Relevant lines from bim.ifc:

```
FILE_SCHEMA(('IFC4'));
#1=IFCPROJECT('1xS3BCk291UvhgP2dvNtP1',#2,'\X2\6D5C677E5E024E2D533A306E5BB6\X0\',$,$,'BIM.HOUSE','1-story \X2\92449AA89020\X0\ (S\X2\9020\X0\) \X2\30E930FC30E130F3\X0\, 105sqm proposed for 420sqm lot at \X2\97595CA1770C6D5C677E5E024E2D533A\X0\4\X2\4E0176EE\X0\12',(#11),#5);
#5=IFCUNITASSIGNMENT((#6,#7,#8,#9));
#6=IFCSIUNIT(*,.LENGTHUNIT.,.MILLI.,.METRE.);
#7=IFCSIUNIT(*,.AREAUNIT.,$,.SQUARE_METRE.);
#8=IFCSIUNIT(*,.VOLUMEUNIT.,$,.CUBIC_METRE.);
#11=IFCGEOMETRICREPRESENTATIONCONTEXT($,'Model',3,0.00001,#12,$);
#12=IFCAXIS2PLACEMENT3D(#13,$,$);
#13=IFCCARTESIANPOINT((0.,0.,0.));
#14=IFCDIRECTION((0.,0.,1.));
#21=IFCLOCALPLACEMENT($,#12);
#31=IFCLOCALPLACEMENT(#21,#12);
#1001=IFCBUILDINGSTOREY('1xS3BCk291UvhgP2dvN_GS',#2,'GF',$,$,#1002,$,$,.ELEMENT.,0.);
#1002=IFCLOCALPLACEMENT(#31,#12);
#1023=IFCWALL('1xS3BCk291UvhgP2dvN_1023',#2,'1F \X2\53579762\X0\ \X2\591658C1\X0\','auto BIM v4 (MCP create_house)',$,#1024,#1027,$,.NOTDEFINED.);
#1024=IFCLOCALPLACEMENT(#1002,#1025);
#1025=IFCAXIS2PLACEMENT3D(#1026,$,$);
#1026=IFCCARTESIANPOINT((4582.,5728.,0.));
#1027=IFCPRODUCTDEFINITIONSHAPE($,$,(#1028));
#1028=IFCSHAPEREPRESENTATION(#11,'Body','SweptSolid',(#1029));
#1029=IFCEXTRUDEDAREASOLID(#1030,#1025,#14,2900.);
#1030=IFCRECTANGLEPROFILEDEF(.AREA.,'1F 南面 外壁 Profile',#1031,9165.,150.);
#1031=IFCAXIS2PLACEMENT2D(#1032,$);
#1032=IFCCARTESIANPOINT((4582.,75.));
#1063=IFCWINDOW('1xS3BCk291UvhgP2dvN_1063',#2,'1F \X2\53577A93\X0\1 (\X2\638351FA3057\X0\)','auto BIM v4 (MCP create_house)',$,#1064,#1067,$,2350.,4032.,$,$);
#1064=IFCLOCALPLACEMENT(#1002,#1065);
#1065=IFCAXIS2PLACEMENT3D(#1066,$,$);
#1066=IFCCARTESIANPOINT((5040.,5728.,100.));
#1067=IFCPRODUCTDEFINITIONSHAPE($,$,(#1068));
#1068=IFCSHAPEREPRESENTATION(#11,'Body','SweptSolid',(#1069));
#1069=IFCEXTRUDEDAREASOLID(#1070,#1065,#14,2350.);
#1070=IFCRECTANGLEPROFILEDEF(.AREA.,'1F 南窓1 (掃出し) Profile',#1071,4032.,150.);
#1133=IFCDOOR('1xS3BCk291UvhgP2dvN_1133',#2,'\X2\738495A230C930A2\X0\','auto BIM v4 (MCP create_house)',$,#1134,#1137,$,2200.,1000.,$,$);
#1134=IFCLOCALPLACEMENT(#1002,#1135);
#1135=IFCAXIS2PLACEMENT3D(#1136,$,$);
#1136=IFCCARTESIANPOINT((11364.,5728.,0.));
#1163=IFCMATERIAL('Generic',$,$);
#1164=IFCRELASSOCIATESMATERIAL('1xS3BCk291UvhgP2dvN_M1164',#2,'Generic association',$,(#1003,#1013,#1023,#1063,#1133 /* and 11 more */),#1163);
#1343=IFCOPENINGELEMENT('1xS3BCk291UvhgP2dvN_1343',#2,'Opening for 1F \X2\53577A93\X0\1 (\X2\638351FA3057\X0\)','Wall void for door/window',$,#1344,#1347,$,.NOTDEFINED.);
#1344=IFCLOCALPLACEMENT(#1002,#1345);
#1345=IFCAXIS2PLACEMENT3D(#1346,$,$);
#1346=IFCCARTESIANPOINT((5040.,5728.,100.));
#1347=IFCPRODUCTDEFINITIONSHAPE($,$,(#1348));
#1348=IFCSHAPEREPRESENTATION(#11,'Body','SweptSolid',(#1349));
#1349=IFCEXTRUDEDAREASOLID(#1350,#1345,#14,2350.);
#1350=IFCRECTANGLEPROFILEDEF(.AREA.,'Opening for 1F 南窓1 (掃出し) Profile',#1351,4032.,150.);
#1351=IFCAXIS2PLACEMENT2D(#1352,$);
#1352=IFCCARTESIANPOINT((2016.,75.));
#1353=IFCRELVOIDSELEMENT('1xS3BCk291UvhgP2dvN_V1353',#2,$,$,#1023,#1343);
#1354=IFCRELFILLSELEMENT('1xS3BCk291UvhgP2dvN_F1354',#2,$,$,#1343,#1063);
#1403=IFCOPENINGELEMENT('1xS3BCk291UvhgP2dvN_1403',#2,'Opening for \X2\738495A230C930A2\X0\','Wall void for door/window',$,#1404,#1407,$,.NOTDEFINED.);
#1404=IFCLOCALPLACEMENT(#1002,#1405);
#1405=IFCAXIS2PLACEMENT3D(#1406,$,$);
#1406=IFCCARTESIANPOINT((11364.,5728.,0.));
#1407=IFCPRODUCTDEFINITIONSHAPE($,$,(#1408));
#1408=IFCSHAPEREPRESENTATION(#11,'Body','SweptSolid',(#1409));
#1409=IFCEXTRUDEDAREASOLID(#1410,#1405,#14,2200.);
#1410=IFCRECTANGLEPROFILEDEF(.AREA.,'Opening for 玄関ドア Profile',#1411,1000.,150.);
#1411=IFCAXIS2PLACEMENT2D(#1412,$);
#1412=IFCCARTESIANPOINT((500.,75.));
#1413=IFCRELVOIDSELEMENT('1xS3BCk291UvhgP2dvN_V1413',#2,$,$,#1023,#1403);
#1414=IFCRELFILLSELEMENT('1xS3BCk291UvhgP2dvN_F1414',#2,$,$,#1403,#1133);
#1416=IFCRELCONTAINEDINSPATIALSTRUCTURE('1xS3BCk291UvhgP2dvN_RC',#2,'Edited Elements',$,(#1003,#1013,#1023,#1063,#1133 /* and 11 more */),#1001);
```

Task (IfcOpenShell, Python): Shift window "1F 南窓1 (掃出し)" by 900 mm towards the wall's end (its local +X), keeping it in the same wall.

```python
import ifcopenshell
import ifcopenshell.api.geometry
import ifcopenshell.util.placement
import ifcopenshell.util.unit

model = ifcopenshell.open("bim.ifc")
unit_scale = ifcopenshell.util.unit.calculate_unit_scale(model)

window = model.by_id(1063)
opening = window.FillsVoids[0].RelatingOpeningElement
wall = opening.VoidsElements[0].RelatingBuildingElement

wall_matrix = ifcopenshell.util.placement.get_local_placement(wall.ObjectPlacement)
shift = wall_matrix[:3, 0] * 0.9 / unit_scale
before = ifcopenshell.util.placement.get_local_placement(window.ObjectPlacement)[:3, 3].copy()

# The window is not placed relative to its opening, so move both.
for product in (opening, window):
    matrix = ifcopenshell.util.placement.get_local_placement(product.ObjectPlacement)
    matrix[:3, 3] += shift
    ifcopenshell.api.geometry.edit_object_placement(model, product=product, matrix=matrix, is_si=False)

after = ifcopenshell.util.placement.get_local_placement(window.ObjectPlacement)[:3, 3]
print("window moved by", (after - before).round(3) + 0.0)

model.write("bim-out.ifc")
```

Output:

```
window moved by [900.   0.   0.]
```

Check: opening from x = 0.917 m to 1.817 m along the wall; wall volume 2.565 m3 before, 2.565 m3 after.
